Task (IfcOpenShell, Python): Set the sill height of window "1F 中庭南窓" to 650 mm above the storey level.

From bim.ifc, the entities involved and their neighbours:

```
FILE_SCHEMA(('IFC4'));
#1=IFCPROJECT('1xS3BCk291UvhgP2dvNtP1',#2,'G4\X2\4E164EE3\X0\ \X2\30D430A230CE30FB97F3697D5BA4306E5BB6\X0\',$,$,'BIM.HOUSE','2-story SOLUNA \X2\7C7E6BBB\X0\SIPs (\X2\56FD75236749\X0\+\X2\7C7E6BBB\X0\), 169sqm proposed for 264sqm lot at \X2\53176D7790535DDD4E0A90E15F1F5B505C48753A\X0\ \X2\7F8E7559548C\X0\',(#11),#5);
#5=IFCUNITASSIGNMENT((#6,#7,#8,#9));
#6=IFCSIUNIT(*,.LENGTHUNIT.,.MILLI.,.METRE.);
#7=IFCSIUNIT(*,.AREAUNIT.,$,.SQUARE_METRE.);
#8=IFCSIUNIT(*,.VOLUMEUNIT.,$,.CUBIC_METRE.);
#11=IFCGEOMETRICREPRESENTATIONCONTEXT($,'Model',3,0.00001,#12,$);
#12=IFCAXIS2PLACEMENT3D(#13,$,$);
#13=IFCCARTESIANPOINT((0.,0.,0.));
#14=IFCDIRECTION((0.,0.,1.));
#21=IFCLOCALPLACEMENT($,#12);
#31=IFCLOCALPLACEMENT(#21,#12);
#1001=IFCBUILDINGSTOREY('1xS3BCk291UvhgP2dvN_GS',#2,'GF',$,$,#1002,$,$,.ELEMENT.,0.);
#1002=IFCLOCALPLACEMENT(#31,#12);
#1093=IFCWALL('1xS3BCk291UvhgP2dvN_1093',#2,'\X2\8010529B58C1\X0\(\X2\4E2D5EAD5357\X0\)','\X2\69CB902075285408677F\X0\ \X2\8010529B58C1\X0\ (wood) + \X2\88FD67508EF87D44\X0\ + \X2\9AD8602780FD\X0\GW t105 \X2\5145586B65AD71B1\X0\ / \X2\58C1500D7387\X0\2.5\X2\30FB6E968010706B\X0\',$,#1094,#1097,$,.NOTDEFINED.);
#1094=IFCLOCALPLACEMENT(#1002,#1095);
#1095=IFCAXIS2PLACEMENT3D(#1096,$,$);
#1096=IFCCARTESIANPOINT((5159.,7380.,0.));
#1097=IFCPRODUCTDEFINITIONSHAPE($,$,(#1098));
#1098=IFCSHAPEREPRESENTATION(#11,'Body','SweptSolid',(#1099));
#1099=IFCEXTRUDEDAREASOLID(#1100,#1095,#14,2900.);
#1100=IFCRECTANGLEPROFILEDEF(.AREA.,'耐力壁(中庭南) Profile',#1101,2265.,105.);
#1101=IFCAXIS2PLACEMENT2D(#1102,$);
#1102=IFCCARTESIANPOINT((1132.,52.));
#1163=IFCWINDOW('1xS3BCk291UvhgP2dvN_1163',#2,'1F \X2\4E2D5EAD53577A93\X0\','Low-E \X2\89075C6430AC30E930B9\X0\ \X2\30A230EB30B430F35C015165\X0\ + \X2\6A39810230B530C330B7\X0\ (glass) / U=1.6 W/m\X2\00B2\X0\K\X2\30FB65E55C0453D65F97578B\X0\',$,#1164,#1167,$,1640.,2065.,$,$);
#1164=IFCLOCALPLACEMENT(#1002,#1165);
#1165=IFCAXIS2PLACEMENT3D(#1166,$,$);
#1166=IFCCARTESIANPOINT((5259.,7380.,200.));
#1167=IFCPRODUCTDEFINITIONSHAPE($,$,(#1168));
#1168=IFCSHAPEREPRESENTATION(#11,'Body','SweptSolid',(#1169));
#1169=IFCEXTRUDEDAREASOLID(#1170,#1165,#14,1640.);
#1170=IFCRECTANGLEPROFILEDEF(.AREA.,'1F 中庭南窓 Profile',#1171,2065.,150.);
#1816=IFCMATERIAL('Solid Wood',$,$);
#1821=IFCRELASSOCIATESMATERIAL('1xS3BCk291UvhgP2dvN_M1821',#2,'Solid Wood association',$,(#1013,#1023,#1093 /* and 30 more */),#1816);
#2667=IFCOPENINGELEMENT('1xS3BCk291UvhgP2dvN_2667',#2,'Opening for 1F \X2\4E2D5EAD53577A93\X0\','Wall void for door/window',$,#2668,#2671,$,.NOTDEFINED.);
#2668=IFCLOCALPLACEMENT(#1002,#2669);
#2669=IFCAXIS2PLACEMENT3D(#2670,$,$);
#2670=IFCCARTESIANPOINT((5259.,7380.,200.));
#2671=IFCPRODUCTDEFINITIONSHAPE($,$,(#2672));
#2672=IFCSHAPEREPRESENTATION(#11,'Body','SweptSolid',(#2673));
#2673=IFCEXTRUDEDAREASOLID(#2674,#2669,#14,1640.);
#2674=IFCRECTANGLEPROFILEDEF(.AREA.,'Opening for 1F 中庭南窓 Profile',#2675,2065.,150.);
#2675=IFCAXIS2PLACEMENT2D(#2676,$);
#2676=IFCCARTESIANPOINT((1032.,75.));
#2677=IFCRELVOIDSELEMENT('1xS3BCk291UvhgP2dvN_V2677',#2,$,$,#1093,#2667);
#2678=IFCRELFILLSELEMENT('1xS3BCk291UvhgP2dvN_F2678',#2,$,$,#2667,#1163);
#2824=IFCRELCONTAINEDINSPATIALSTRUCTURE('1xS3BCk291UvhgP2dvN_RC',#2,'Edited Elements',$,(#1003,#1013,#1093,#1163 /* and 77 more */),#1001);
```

```python
import numpy as np
import ifcopenshell
import ifcopenshell.api.geometry
import ifcopenshell.geom
import ifcopenshell.util.element
import ifcopenshell.util.placement
import ifcopenshell.util.shape
import ifcopenshell.util.unit

model = ifcopenshell.open("bim.ifc")
unit_scale = ifcopenshell.util.unit.calculate_unit_scale(model)

window = model.by_id(1163)
opening = window.FillsVoids[0].RelatingOpeningElement
storey = ifcopenshell.util.element.get_container(window, ifc_class="IfcBuildingStorey")
level = ifcopenshell.util.placement.get_local_placement(storey.ObjectPlacement)[2, 3]

# The opening's origin need not be at the sill, so measure its lowest point.
shape = ifcopenshell.geom.create_shape(ifcopenshell.geom.settings(), opening)
bottom = ifcopenshell.util.shape.get_shape_bottom_elevation(shape, shape.geometry) / unit_scale
dz = level + 0.65 / unit_scale - bottom

shift = np.array([0.0, 0.0, dz])
# The window is not placed relative to its opening, so move both.
for product in (opening, window):
    matrix = ifcopenshell.util.placement.get_local_placement(product.ObjectPlacement)
    matrix[:3, 3] += shift
    ifcopenshell.api.geometry.edit_object_placement(model, product=product, matrix=matrix, is_si=False)

print(f"moved by {dz * unit_scale:+.3f} m")

model.write("bim_v2.ifc")
```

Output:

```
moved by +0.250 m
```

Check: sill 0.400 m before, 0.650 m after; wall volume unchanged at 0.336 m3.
